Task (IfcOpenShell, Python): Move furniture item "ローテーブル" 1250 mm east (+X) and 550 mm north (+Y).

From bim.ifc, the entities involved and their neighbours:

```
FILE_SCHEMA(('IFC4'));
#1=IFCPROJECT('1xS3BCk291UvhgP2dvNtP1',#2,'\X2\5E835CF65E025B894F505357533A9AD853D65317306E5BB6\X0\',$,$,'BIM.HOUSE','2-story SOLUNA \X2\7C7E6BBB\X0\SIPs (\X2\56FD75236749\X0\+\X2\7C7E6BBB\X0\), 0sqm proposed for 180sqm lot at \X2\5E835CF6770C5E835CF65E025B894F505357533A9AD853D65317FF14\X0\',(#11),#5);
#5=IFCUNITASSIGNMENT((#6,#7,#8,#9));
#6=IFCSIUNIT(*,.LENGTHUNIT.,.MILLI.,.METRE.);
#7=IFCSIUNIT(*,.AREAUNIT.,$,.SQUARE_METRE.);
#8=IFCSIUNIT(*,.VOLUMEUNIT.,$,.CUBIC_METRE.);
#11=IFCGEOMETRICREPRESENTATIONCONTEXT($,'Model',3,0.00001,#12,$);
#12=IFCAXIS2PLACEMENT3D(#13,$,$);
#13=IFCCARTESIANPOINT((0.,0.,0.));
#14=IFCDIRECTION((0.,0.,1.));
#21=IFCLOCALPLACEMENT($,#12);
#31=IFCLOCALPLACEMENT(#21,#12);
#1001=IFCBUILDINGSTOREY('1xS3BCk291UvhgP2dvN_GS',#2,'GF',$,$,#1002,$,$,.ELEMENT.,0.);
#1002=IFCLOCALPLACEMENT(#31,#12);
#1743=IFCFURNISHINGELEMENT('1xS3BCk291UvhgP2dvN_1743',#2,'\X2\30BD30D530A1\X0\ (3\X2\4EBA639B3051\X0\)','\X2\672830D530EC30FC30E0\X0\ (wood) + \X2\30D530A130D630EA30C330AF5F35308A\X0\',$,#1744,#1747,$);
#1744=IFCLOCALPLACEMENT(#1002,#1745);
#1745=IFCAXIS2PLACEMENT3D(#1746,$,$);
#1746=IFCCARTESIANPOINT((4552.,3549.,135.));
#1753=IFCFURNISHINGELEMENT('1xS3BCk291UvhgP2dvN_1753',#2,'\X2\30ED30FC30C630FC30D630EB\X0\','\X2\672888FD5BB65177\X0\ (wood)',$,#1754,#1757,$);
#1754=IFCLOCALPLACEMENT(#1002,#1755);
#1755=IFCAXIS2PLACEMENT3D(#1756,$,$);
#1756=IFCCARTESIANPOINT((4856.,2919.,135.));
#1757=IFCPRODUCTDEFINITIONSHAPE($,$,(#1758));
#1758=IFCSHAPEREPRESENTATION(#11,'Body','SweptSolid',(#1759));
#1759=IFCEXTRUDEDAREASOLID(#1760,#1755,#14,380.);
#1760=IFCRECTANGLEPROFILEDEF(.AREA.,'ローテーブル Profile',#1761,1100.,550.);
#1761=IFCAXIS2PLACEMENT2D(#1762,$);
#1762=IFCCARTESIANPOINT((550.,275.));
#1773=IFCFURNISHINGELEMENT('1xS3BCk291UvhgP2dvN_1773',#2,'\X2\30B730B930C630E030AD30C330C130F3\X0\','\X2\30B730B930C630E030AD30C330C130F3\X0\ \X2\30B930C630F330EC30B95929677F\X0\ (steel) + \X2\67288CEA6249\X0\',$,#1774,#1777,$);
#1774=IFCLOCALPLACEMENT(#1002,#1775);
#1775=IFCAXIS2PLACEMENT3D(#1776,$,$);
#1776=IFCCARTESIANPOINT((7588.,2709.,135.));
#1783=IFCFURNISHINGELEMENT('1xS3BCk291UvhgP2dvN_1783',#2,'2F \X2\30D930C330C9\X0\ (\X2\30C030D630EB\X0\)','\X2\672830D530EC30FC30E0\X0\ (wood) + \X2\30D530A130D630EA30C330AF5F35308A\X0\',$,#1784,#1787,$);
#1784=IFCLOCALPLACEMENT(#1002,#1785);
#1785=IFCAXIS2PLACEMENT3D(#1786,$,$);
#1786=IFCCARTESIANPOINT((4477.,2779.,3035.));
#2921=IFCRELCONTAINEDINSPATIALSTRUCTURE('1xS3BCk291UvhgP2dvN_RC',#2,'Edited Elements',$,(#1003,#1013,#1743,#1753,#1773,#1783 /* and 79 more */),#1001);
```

```python
import ifcopenshell
import ifcopenshell.api.geometry
import ifcopenshell.util.placement
import ifcopenshell.util.unit

model = ifcopenshell.open("bim.ifc")
unit_scale = ifcopenshell.util.unit.calculate_unit_scale(model)

item = model.by_guid("1xS3BCk291UvhgP2dvN_1753")
matrix = ifcopenshell.util.placement.get_local_placement(item.ObjectPlacement)
matrix[0, 3] += 1.25 / unit_scale
matrix[1, 3] += 0.55 / unit_scale
ifcopenshell.api.geometry.edit_object_placement(model, product=item, matrix=matrix, is_si=False)

print(ifcopenshell.util.placement.get_local_placement(item.ObjectPlacement).round(3) + 0.0)

model.write("bim_updated.ifc")
```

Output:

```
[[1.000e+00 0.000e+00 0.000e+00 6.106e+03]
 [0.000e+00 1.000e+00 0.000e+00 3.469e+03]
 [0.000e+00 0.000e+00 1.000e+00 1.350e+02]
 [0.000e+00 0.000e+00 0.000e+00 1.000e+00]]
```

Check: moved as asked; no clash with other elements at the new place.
